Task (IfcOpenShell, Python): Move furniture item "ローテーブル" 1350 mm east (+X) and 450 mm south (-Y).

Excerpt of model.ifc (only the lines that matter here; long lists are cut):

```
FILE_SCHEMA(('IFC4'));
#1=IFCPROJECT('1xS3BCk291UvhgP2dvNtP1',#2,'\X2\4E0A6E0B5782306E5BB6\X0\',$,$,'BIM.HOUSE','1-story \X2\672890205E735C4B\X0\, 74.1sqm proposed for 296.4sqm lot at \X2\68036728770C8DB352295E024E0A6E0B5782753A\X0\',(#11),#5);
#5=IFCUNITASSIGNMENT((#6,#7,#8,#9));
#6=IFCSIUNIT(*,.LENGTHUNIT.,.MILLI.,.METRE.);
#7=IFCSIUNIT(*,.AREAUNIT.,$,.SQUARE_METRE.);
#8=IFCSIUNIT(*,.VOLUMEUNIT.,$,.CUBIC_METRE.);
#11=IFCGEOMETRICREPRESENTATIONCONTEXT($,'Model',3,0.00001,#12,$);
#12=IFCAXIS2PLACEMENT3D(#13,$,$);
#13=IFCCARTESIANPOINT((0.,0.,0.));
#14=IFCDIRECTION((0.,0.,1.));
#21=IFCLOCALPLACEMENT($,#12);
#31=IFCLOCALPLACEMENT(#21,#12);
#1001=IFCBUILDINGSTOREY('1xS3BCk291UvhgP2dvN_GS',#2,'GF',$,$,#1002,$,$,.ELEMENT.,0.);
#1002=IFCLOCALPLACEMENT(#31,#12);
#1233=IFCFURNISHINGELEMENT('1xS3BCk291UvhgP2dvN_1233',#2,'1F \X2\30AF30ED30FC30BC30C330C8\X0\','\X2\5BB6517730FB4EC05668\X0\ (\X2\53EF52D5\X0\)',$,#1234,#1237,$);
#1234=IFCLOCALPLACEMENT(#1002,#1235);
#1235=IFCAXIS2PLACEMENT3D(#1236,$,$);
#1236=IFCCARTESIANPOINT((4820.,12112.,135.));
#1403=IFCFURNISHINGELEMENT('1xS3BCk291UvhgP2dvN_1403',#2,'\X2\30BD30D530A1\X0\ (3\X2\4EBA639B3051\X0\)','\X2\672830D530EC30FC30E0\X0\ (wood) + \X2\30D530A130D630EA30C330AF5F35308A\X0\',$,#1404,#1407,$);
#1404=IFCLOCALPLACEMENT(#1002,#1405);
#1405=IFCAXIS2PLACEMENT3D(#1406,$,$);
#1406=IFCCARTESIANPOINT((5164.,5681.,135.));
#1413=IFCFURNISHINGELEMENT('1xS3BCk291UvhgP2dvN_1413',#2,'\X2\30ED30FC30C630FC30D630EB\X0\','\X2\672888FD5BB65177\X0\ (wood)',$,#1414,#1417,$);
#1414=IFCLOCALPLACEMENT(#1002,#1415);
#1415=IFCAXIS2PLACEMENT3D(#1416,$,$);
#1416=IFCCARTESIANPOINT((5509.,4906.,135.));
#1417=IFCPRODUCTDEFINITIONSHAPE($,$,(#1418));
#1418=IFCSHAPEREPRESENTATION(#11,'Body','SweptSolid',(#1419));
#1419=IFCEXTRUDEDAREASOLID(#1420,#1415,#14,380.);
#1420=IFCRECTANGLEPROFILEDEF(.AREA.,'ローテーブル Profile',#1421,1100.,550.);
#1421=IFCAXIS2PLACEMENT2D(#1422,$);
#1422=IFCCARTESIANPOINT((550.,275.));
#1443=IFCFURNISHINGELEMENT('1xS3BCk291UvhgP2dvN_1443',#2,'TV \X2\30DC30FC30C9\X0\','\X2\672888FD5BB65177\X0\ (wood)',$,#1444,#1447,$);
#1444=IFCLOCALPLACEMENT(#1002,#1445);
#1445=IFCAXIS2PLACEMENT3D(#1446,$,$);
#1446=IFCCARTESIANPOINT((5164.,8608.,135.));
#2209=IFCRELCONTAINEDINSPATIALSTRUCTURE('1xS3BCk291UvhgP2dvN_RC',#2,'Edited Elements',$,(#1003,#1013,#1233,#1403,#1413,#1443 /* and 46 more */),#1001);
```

```python
import ifcopenshell
import ifcopenshell.api.geometry
import ifcopenshell.util.placement

model = ifcopenshell.open("model.ifc")

item = model.by_guid("1xS3BCk291UvhgP2dvN_1413")
matrix = ifcopenshell.util.placement.get_local_placement(item.ObjectPlacement)
matrix[0, 3] += 1350.0
matrix[1, 3] -= 450.0
ifcopenshell.api.geometry.edit_object_placement(model, product=item, matrix=matrix, is_si=False)

print(ifcopenshell.util.placement.get_local_placement(item.ObjectPlacement).round(3) + 0.0)

model.write("model-out.ifc")
```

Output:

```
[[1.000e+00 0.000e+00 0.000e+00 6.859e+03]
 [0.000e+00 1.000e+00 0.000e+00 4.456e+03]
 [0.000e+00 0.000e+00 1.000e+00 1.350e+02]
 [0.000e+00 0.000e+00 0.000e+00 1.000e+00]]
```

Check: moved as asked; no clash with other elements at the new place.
